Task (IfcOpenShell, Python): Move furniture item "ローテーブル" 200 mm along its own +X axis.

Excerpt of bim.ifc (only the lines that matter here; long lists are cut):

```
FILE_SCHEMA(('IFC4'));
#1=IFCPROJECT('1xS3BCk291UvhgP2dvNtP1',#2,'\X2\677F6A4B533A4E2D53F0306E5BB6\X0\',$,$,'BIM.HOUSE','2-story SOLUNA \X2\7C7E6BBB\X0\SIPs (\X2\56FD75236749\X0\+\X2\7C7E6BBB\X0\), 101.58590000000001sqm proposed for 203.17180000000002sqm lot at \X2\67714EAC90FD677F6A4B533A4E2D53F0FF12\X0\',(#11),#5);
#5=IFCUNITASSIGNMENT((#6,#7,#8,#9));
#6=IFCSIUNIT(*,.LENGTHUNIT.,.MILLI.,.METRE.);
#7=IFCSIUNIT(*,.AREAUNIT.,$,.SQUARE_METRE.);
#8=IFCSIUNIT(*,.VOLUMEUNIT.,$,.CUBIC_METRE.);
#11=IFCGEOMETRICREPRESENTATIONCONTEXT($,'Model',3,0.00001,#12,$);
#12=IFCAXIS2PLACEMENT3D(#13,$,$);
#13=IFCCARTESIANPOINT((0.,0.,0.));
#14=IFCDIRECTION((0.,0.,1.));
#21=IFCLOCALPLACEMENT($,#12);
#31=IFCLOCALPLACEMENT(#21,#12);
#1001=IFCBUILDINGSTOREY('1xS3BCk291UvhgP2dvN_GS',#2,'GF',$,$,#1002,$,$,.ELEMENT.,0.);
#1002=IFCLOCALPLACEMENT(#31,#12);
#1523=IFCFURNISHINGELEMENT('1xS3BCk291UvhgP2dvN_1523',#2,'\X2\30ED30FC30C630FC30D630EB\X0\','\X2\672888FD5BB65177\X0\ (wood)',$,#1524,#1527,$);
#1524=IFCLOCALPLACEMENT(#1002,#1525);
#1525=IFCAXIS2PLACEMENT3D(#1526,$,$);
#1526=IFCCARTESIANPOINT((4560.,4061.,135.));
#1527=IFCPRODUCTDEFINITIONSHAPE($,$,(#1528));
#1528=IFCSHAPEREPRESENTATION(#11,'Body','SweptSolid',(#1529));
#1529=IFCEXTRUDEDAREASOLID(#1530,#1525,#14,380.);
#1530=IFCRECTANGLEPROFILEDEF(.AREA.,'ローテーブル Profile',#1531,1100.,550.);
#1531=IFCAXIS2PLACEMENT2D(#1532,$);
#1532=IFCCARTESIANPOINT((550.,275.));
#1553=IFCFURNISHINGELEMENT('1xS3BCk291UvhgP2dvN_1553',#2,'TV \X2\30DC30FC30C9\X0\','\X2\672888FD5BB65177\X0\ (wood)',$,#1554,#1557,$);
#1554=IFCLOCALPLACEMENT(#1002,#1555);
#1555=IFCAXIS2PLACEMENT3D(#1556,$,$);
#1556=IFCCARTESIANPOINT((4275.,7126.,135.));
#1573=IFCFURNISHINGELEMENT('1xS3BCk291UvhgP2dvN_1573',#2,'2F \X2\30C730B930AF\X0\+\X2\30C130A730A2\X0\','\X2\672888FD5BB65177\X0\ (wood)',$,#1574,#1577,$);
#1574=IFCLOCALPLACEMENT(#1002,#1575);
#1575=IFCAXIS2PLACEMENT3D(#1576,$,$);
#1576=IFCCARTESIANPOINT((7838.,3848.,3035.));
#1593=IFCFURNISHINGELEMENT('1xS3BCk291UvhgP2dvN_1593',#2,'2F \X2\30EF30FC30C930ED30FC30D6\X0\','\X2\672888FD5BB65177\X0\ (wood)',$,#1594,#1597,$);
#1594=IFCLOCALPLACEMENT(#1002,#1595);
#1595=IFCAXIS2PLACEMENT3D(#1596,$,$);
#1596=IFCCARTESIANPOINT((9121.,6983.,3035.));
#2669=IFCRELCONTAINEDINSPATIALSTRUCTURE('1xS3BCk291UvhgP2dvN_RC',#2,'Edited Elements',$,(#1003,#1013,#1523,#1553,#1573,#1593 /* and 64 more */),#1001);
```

```python
import ifcopenshell
import ifcopenshell.api.geometry
import ifcopenshell.util.placement

model = ifcopenshell.open("bim.ifc")

item = model.by_id(1523)
matrix = ifcopenshell.util.placement.get_local_placement(item.ObjectPlacement)
matrix[:3, 3] += matrix[:3, 0] * 200.0
ifcopenshell.api.geometry.edit_object_placement(model, product=item, matrix=matrix, is_si=False)

print(ifcopenshell.util.placement.get_local_placement(item.ObjectPlacement).round(3) + 0.0)

model.write("bim-out.ifc")
```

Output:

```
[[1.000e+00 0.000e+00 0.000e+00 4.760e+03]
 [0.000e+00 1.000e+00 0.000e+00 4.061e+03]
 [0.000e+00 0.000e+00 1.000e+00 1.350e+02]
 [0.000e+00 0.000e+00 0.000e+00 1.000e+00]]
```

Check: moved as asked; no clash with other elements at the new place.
